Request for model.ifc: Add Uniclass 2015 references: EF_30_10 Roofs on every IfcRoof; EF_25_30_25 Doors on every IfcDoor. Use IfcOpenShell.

First a look at what the model holds.

```python
import ifcopenshell

model = ifcopenshell.open("model.ifc")
print(model.schema)
print("classifications:", [c.Name for c in model.by_type("IfcClassification")])
for ifc_class in ("IfcDoor", "IfcRoof", "IfcStair", "IfcWall", "IfcWindow"):
    print(ifc_class, len(model.by_type(ifc_class)))
```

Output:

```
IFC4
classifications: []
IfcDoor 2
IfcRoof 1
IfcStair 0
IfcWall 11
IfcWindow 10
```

```python
import ifcopenshell
import ifcopenshell.api.classification

model = ifcopenshell.open("model.ifc")

system = ifcopenshell.api.classification.add_classification(model, classification="Uniclass 2015")

codes = {
    "IfcRoof": ("EF_30_10", "Roofs"),
    "IfcDoor": ("EF_25_30_25", "Doors"),
}
for ifc_class, (code, name) in codes.items():
    products = model.by_type(ifc_class)
    ifcopenshell.api.classification.add_reference(
        model, products=products, classification=system, identification=code, name=name
    )
    print(code, len(products))

model.write("model_edited.ifc")
```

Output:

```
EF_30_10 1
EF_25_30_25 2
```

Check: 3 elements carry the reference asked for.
